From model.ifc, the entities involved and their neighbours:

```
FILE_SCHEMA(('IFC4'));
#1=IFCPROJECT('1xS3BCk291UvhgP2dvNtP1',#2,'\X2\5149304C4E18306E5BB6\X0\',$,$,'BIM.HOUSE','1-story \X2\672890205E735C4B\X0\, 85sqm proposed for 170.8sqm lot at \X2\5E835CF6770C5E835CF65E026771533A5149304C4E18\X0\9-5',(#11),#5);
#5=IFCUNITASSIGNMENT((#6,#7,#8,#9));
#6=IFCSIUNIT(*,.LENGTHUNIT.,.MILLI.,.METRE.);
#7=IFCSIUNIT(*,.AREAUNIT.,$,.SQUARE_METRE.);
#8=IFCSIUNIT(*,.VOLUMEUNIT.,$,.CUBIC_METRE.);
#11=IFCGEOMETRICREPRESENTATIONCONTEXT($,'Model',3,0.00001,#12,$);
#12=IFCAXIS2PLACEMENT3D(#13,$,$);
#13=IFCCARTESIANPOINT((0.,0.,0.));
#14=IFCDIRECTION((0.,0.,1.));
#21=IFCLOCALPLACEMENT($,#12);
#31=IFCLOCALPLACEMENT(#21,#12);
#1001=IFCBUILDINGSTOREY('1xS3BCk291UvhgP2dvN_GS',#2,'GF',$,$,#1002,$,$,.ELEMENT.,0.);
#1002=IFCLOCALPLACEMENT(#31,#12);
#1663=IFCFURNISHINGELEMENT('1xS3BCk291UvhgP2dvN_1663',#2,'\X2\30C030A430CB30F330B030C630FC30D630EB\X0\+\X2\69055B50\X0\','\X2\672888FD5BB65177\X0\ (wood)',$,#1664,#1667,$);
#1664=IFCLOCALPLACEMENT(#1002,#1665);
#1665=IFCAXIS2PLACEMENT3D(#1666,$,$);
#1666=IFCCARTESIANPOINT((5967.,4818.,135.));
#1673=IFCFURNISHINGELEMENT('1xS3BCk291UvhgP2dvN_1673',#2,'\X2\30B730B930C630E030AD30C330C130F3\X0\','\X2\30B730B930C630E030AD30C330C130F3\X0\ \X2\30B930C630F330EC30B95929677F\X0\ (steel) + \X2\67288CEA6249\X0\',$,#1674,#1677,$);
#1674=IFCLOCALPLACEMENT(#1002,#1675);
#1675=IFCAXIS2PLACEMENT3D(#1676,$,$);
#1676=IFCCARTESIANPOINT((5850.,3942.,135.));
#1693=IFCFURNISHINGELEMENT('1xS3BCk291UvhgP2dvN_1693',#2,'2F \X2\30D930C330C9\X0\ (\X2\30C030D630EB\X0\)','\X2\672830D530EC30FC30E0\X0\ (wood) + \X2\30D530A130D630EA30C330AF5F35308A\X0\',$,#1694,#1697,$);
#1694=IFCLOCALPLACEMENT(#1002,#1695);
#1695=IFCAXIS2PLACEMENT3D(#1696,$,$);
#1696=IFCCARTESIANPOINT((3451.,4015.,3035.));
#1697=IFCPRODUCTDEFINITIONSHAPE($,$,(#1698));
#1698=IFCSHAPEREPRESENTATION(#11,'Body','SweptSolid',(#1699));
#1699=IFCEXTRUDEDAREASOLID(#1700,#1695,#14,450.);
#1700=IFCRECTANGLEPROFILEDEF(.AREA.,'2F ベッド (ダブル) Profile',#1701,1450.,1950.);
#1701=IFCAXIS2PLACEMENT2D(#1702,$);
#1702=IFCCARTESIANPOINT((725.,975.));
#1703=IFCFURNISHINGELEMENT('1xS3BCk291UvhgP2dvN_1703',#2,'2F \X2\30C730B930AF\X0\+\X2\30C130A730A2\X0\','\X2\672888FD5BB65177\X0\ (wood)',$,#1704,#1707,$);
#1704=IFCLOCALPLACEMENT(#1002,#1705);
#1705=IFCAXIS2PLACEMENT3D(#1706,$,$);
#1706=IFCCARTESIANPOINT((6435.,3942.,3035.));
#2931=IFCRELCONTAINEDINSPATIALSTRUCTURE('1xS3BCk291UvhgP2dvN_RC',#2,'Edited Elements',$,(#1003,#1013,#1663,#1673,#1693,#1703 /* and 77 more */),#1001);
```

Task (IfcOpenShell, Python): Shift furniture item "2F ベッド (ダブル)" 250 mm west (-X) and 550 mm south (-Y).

```python
import ifcopenshell
import ifcopenshell.api.geometry
import ifcopenshell.util.placement
import ifcopenshell.util.unit

model = ifcopenshell.open("model.ifc")
unit_scale = ifcopenshell.util.unit.calculate_unit_scale(model)

item = model.by_guid("1xS3BCk291UvhgP2dvN_1693")
matrix = ifcopenshell.util.placement.get_local_placement(item.ObjectPlacement)
matrix[0, 3] -= 0.25 / unit_scale
matrix[1, 3] -= 0.55 / unit_scale
ifcopenshell.api.geometry.edit_object_placement(model, product=item, matrix=matrix, is_si=False)

print(ifcopenshell.util.placement.get_local_placement(item.ObjectPlacement).round(3) + 0.0)

model.write("model_v2.ifc")
```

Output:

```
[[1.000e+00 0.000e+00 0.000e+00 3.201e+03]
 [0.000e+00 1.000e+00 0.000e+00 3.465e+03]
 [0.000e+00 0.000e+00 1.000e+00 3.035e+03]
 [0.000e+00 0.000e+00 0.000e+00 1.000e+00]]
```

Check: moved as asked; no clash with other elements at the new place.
